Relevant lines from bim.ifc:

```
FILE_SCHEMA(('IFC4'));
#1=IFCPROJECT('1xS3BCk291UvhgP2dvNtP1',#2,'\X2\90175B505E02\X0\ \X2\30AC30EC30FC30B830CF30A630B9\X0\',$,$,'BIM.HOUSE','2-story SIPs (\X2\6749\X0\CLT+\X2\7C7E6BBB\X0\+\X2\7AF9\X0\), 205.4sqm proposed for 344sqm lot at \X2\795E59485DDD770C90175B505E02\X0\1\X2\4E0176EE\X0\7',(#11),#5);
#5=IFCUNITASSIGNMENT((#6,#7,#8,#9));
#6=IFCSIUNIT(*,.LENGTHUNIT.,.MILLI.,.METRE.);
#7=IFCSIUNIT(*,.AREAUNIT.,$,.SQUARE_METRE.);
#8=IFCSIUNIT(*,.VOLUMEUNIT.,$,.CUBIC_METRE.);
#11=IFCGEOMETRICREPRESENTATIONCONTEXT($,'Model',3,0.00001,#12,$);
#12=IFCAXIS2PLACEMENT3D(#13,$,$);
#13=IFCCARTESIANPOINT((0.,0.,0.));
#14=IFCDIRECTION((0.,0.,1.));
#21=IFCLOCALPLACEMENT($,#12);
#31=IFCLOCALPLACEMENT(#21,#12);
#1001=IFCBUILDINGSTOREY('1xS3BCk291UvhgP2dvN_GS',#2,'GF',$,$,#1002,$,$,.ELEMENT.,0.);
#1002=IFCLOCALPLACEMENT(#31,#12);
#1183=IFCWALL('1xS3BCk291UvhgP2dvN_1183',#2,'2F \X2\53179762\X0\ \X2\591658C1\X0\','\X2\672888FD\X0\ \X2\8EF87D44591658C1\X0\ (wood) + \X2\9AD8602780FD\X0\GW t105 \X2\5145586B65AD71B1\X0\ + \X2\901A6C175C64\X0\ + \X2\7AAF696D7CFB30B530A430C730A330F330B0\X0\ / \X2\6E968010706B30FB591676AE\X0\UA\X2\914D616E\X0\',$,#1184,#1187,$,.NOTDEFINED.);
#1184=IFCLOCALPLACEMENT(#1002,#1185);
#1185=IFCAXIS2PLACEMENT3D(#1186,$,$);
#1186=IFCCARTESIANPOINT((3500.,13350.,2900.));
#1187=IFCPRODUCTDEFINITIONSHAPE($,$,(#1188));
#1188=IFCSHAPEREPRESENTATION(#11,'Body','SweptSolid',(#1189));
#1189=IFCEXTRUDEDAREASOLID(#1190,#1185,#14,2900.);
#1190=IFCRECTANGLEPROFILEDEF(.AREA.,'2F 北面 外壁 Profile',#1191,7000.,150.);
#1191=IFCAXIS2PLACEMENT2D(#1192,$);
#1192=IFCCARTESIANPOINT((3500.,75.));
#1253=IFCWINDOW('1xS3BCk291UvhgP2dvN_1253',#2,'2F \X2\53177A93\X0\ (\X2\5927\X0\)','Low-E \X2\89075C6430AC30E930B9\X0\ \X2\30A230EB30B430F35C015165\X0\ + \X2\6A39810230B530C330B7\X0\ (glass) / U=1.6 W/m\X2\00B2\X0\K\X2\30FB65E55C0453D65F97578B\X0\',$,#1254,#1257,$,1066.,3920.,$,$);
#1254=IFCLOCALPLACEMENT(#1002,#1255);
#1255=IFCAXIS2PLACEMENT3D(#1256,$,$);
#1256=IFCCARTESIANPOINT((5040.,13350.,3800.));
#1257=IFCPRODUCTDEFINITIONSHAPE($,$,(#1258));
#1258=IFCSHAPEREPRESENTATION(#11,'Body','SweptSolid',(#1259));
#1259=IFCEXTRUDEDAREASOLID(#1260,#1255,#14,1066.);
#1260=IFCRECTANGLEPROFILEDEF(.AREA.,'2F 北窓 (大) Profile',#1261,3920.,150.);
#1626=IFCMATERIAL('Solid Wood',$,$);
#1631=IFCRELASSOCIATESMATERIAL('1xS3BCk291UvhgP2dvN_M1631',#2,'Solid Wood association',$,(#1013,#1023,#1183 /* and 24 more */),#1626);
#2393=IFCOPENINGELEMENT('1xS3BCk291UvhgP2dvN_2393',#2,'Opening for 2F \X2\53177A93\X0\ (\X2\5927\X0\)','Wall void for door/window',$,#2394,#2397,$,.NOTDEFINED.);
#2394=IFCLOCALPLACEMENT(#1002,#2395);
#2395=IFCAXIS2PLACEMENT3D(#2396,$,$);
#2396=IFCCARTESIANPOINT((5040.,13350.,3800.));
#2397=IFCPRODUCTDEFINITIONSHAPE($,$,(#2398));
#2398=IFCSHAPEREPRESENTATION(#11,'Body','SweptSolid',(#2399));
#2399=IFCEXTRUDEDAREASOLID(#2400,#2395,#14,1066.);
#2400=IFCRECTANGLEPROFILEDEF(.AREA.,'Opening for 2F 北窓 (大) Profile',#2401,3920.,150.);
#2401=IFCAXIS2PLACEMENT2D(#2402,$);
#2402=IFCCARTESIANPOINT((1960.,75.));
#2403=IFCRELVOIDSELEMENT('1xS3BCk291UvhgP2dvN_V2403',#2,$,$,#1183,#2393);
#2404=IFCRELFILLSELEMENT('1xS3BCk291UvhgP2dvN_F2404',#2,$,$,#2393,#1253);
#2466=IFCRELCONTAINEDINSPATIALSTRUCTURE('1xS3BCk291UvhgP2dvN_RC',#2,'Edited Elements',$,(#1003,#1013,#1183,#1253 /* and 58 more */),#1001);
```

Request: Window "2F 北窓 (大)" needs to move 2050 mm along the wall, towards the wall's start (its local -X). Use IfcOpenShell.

```python
import ifcopenshell
import ifcopenshell.api.geometry
import ifcopenshell.util.placement
import ifcopenshell.util.unit

model = ifcopenshell.open("bim.ifc")
unit_scale = ifcopenshell.util.unit.calculate_unit_scale(model)

window = model.by_guid("1xS3BCk291UvhgP2dvN_1253")
opening = window.FillsVoids[0].RelatingOpeningElement
wall = opening.VoidsElements[0].RelatingBuildingElement

wall_matrix = ifcopenshell.util.placement.get_local_placement(wall.ObjectPlacement)
shift = wall_matrix[:3, 0] * -2.05 / unit_scale
before = ifcopenshell.util.placement.get_local_placement(window.ObjectPlacement)[:3, 3].copy()

# The window is not placed relative to its opening, so move both.
for product in (opening, window):
    matrix = ifcopenshell.util.placement.get_local_placement(product.ObjectPlacement)
    matrix[:3, 3] += shift
    ifcopenshell.api.geometry.edit_object_placement(model, product=product, matrix=matrix, is_si=False)

after = ifcopenshell.util.placement.get_local_placement(window.ObjectPlacement)[:3, 3]
print("window moved by", (after - before).round(3) + 0.0)

model.write("bim_v2.ifc")
```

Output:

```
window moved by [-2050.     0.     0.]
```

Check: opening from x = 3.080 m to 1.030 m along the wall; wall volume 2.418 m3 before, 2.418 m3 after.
